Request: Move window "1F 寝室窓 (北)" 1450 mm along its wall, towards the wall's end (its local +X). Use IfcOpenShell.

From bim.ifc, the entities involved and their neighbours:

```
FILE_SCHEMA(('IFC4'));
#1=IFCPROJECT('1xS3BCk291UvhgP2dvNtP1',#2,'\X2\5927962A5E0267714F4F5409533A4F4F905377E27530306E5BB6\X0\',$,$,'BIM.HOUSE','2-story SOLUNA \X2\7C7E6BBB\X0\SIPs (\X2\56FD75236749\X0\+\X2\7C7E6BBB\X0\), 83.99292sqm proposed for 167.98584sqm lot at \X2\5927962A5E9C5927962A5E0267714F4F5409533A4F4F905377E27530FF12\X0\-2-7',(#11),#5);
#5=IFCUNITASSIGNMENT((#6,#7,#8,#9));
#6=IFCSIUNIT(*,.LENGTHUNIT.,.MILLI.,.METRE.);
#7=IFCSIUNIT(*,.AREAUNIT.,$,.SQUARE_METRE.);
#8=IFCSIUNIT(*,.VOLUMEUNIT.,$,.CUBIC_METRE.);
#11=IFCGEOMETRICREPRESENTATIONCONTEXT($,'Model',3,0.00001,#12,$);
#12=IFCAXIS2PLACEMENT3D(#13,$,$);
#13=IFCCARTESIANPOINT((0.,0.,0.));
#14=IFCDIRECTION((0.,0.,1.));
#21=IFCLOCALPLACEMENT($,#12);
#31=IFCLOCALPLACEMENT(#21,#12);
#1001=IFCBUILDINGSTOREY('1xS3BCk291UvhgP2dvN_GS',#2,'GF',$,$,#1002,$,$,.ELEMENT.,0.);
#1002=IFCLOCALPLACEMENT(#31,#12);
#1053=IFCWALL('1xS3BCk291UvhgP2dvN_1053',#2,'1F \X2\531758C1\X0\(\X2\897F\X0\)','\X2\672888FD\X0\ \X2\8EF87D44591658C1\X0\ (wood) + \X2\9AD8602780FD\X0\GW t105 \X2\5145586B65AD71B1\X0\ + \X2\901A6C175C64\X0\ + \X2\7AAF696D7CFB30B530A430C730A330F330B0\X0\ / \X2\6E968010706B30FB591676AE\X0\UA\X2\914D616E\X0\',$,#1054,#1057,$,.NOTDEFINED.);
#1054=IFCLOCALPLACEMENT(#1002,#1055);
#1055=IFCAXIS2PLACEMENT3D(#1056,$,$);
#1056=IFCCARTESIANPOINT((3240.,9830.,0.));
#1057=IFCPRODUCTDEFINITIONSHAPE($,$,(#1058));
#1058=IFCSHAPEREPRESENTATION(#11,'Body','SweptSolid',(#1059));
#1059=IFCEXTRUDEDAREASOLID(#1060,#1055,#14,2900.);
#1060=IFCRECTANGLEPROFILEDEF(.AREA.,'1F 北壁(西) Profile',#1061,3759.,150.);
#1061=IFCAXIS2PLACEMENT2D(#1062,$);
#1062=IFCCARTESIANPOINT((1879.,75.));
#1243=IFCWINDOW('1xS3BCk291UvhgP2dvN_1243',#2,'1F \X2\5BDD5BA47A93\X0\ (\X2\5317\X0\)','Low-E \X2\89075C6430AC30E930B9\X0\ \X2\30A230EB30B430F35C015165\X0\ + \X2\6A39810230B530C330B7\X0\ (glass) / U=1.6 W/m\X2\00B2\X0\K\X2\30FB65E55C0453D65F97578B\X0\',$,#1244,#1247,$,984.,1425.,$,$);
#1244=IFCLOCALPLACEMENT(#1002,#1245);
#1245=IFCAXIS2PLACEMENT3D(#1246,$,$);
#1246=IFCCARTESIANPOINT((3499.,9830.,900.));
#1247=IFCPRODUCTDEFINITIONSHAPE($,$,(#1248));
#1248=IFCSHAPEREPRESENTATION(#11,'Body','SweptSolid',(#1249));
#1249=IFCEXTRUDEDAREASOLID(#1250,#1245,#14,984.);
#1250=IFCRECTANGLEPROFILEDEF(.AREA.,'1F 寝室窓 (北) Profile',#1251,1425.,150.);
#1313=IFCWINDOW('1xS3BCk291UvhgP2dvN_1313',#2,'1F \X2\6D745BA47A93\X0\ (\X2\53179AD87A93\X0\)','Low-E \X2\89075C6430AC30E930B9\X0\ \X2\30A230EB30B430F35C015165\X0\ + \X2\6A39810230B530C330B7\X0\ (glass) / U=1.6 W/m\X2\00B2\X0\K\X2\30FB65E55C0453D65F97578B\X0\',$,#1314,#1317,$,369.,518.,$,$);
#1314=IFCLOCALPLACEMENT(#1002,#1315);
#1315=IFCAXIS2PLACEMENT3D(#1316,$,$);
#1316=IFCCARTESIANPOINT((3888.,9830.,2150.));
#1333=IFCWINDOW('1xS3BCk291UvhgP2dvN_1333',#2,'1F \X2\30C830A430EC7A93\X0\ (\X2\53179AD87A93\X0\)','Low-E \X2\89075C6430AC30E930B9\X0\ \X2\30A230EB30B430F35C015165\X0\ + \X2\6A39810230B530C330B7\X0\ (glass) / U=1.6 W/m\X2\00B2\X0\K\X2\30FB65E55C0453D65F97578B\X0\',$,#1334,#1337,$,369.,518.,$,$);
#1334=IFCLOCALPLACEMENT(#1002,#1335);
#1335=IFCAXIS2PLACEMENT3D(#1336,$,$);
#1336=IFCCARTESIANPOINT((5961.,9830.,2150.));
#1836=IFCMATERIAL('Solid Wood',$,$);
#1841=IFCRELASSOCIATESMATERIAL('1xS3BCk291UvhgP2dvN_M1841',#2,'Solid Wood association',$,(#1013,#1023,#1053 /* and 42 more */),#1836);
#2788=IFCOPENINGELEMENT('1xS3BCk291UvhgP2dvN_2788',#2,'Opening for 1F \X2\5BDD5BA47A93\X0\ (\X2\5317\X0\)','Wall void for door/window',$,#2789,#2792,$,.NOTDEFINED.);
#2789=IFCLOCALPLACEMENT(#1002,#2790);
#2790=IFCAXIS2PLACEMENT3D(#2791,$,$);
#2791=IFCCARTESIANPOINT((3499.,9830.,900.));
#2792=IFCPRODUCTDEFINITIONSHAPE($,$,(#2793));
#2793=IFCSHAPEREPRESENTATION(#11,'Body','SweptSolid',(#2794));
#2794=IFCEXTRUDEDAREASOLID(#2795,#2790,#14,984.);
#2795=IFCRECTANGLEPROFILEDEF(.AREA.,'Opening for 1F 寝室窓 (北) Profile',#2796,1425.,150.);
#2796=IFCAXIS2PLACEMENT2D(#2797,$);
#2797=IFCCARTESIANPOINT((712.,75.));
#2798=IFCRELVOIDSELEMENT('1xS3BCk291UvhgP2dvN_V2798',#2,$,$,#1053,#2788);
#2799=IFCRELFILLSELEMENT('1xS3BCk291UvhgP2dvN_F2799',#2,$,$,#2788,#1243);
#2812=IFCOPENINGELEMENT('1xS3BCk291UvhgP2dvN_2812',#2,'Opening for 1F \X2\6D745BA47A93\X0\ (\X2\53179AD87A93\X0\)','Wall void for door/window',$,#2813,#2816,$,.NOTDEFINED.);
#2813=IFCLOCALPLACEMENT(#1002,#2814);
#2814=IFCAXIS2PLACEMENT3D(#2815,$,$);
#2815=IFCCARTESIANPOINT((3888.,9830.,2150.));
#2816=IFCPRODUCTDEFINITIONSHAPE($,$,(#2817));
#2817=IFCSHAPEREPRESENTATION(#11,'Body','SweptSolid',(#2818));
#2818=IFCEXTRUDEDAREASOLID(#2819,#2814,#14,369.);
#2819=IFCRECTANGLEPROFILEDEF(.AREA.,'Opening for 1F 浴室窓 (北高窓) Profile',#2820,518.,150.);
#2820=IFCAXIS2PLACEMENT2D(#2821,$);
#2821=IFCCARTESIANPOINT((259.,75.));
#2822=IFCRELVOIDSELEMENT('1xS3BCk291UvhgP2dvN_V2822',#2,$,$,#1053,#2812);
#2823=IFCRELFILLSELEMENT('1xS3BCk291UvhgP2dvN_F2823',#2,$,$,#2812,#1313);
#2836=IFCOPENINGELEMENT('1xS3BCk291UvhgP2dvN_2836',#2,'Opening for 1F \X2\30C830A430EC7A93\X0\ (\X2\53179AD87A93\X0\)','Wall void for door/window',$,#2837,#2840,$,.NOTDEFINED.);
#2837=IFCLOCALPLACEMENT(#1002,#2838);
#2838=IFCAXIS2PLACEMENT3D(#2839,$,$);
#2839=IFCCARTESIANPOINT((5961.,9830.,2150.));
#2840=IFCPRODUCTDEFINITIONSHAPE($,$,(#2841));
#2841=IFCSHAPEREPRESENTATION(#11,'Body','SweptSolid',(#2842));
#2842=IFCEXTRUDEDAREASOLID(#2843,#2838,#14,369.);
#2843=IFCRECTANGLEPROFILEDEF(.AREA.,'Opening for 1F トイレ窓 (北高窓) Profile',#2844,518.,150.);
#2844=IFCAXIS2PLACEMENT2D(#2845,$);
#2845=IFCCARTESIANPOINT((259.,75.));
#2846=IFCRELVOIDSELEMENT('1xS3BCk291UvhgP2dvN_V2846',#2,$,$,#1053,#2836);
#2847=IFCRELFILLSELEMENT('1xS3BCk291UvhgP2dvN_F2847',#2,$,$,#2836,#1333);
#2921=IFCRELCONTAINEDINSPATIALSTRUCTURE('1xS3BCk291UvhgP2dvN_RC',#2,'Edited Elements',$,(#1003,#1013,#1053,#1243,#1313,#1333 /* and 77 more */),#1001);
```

```python
import ifcopenshell
import ifcopenshell.api.geometry
import ifcopenshell.util.placement
import ifcopenshell.util.unit

model = ifcopenshell.open("bim.ifc")
unit_scale = ifcopenshell.util.unit.calculate_unit_scale(model)

window = model.by_id(1243)
opening = window.FillsVoids[0].RelatingOpeningElement
wall = opening.VoidsElements[0].RelatingBuildingElement

wall_matrix = ifcopenshell.util.placement.get_local_placement(wall.ObjectPlacement)
shift = wall_matrix[:3, 0] * 1.45 / unit_scale
before = ifcopenshell.util.placement.get_local_placement(window.ObjectPlacement)[:3, 3].copy()

# The window is not placed relative to its opening, so move both.
for product in (opening, window):
    matrix = ifcopenshell.util.placement.get_local_placement(product.ObjectPlacement)
    matrix[:3, 3] += shift
    ifcopenshell.api.geometry.edit_object_placement(model, product=product, matrix=matrix, is_si=False)

after = ifcopenshell.util.placement.get_local_placement(window.ObjectPlacement)[:3, 3]
print("window moved by", (after - before).round(3) + 0.0)

model.write("bim_updated.ifc")
```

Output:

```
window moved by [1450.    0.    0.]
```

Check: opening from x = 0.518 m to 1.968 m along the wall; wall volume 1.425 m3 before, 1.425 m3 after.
